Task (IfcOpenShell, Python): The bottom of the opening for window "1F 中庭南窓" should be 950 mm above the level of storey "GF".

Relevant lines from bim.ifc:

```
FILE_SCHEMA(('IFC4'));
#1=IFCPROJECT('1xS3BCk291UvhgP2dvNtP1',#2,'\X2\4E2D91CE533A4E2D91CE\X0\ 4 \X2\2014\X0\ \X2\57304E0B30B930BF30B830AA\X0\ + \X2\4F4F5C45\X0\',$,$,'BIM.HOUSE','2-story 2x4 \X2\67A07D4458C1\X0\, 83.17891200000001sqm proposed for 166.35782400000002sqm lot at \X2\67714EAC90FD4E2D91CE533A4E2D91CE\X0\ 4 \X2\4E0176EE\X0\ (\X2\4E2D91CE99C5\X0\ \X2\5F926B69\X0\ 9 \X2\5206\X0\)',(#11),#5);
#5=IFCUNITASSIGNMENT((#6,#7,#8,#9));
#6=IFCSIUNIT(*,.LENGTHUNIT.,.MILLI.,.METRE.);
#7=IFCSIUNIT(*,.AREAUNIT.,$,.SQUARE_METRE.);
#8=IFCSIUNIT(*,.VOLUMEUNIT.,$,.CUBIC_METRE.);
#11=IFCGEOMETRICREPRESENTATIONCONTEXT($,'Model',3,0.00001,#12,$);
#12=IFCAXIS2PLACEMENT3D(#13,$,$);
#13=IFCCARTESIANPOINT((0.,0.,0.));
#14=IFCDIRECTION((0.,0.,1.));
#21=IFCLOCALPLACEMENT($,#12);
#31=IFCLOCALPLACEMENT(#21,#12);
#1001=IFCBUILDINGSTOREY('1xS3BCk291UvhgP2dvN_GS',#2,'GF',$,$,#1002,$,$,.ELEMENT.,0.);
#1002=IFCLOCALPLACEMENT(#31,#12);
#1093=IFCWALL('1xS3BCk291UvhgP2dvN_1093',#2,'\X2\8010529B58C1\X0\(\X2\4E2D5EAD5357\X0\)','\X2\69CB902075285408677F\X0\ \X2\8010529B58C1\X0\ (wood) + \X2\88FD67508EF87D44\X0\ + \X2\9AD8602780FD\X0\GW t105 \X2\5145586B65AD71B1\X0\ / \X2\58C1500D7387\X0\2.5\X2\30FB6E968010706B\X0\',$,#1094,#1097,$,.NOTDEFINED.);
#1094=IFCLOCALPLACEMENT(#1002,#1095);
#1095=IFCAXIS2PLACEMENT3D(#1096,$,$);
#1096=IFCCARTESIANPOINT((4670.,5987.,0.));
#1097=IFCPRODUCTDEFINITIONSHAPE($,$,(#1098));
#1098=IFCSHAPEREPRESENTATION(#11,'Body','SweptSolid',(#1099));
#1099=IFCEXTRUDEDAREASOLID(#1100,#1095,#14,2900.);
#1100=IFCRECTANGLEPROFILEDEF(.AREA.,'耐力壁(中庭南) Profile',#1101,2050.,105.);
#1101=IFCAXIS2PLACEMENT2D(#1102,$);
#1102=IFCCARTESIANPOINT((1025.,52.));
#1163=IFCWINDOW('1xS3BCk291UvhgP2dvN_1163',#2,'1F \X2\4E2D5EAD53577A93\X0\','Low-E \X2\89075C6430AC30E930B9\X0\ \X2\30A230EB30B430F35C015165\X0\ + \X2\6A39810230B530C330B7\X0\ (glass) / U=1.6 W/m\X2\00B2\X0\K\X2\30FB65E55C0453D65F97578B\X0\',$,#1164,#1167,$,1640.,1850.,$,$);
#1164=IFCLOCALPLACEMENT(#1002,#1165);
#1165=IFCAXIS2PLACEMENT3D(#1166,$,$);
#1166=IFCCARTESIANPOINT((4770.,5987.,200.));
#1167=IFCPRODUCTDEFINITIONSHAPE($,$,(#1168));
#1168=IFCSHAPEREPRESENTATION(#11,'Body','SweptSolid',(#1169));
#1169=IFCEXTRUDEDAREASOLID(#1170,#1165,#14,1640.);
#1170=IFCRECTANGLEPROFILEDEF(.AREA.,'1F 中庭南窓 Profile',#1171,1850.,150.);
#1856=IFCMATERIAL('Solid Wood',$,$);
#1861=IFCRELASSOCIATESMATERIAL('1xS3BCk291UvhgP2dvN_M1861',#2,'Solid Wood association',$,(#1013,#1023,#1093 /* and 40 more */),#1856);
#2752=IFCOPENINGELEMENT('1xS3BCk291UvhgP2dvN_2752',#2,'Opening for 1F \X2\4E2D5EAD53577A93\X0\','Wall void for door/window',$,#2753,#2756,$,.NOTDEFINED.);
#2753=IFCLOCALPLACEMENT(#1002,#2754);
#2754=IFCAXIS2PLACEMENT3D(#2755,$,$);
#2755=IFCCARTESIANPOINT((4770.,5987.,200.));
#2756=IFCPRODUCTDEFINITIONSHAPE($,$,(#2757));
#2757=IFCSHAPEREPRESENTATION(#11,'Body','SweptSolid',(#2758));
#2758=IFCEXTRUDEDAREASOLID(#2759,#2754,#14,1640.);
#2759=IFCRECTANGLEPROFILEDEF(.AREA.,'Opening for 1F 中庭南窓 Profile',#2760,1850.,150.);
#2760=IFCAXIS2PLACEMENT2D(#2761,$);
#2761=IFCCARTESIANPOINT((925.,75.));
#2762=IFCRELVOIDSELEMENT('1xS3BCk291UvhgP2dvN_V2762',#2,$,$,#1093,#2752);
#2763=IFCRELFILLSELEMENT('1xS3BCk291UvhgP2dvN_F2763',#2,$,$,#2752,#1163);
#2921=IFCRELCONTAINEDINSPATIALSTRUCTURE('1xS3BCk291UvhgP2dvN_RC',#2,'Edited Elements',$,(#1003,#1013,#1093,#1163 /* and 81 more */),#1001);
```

```python
import numpy as np
import ifcopenshell
import ifcopenshell.api.geometry
import ifcopenshell.geom
import ifcopenshell.util.element
import ifcopenshell.util.placement
import ifcopenshell.util.shape
import ifcopenshell.util.unit

model = ifcopenshell.open("bim.ifc")
unit_scale = ifcopenshell.util.unit.calculate_unit_scale(model)

window = model.by_guid("1xS3BCk291UvhgP2dvN_1163")
opening = window.FillsVoids[0].RelatingOpeningElement
storey = ifcopenshell.util.element.get_container(window, ifc_class="IfcBuildingStorey")
level = ifcopenshell.util.placement.get_local_placement(storey.ObjectPlacement)[2, 3]

# The opening's origin need not be at the sill, so measure its lowest point.
shape = ifcopenshell.geom.create_shape(ifcopenshell.geom.settings(), opening)
bottom = ifcopenshell.util.shape.get_shape_bottom_elevation(shape, shape.geometry) / unit_scale
dz = level + 950.0 - bottom

shift = np.array([0.0, 0.0, dz])
# The window is not placed relative to its opening, so move both.
for product in (opening, window):
    matrix = ifcopenshell.util.placement.get_local_placement(product.ObjectPlacement)
    matrix[:3, 3] += shift
    ifcopenshell.api.geometry.edit_object_placement(model, product=product, matrix=matrix, is_si=False)

print(f"moved by {dz * unit_scale:+.3f} m")

model.write("bim_rev.ifc")
```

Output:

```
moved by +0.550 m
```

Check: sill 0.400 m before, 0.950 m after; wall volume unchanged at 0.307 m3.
